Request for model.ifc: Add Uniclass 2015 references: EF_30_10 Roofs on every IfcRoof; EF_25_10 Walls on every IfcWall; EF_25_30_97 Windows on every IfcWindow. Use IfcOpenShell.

First a look at what the model holds.

```python
import ifcopenshell

model = ifcopenshell.open("model.ifc")
print(model.schema)
print("classifications:", [c.Name for c in model.by_type("IfcClassification")])
for ifc_class in ("IfcDoor", "IfcRoof", "IfcStair", "IfcWall", "IfcWindow"):
    print(ifc_class, len(model.by_type(ifc_class)))
```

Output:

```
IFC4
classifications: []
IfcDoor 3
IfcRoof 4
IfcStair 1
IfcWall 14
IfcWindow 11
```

```python
import ifcopenshell
import ifcopenshell.api.classification

model = ifcopenshell.open("model.ifc")

system = ifcopenshell.api.classification.add_classification(model, classification="Uniclass 2015")

codes = {
    "IfcRoof": ("EF_30_10", "Roofs"),
    "IfcWall": ("EF_25_10", "Walls"),
    "IfcWindow": ("EF_25_30_97", "Windows"),
}
for ifc_class, (code, name) in codes.items():
    products = model.by_type(ifc_class)
    ifcopenshell.api.classification.add_reference(
        model, products=products, classification=system, identification=code, name=name
    )
    print(code, len(products))

model.write("model-out.ifc")
```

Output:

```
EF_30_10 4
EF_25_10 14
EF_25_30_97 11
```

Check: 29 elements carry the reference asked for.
